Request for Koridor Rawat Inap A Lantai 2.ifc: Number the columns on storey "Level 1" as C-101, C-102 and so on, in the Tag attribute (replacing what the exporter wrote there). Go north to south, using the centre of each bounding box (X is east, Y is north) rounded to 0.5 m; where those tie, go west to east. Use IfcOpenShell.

First a look at what the model holds.

```python
import ifcopenshell
import ifcopenshell.util.element
import ifcopenshell.util.placement

model = ifcopenshell.open("Koridor Rawat Inap A Lantai 2.ifc")
print(model.schema)
storey = next(s for s in model.by_type("IfcBuildingStorey") if s.Name == "Level 1")
columns = [e for e in ifcopenshell.util.element.get_decomposition(storey) if e.is_a("IfcColumn")]
for e in sorted(columns, key=lambda e: e.id()):
    origin = ifcopenshell.util.placement.get_local_placement(e.ObjectPlacement)[:3, 3]
    print(e.id(), e.Tag, e.Name, origin.round(2) + 0.0, sep=" | ")
```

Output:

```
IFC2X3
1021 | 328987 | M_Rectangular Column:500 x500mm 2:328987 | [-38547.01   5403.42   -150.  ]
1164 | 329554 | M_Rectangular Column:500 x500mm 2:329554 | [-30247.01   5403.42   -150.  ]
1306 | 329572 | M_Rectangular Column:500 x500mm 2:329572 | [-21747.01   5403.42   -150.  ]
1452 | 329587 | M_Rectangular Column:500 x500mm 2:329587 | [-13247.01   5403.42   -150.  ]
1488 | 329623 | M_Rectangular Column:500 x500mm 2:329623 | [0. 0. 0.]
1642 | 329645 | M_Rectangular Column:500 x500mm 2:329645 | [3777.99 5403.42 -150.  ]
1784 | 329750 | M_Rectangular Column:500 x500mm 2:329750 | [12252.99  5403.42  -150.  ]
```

```python
import ifcopenshell
import ifcopenshell.geom
import ifcopenshell.util.element
import ifcopenshell.util.shape

model = ifcopenshell.open("Koridor Rawat Inap A Lantai 2.ifc")
settings = ifcopenshell.geom.settings()
settings.set("use-world-coords", True)


def centre(element):
    shape = ifcopenshell.geom.create_shape(settings, element)
    return ifcopenshell.util.shape.get_bbox_centroid(shape.geometry)


storey = next(s for s in model.by_type("IfcBuildingStorey") if s.Name == "Level 1")
columns = [e for e in ifcopenshell.util.element.get_decomposition(storey) if e.is_a("IfcColumn")]

# Insertion points can sit at a corner or the storey origin, so sort by the geometry (in metres).
centres = {e: centre(e) for e in columns}
columns.sort(key=lambda e: (-round(centres[e][1] / 0.5), centres[e][0]))

for i, e in enumerate(columns, start=1):
    number = f"C-1{i:02d}"
    e.Tag = number
    print(e.id(), number)

model.write("Koridor Rawat Inap A Lantai 2_v2.ifc")
```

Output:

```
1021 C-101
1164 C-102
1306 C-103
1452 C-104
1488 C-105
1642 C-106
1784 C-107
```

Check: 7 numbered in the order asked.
